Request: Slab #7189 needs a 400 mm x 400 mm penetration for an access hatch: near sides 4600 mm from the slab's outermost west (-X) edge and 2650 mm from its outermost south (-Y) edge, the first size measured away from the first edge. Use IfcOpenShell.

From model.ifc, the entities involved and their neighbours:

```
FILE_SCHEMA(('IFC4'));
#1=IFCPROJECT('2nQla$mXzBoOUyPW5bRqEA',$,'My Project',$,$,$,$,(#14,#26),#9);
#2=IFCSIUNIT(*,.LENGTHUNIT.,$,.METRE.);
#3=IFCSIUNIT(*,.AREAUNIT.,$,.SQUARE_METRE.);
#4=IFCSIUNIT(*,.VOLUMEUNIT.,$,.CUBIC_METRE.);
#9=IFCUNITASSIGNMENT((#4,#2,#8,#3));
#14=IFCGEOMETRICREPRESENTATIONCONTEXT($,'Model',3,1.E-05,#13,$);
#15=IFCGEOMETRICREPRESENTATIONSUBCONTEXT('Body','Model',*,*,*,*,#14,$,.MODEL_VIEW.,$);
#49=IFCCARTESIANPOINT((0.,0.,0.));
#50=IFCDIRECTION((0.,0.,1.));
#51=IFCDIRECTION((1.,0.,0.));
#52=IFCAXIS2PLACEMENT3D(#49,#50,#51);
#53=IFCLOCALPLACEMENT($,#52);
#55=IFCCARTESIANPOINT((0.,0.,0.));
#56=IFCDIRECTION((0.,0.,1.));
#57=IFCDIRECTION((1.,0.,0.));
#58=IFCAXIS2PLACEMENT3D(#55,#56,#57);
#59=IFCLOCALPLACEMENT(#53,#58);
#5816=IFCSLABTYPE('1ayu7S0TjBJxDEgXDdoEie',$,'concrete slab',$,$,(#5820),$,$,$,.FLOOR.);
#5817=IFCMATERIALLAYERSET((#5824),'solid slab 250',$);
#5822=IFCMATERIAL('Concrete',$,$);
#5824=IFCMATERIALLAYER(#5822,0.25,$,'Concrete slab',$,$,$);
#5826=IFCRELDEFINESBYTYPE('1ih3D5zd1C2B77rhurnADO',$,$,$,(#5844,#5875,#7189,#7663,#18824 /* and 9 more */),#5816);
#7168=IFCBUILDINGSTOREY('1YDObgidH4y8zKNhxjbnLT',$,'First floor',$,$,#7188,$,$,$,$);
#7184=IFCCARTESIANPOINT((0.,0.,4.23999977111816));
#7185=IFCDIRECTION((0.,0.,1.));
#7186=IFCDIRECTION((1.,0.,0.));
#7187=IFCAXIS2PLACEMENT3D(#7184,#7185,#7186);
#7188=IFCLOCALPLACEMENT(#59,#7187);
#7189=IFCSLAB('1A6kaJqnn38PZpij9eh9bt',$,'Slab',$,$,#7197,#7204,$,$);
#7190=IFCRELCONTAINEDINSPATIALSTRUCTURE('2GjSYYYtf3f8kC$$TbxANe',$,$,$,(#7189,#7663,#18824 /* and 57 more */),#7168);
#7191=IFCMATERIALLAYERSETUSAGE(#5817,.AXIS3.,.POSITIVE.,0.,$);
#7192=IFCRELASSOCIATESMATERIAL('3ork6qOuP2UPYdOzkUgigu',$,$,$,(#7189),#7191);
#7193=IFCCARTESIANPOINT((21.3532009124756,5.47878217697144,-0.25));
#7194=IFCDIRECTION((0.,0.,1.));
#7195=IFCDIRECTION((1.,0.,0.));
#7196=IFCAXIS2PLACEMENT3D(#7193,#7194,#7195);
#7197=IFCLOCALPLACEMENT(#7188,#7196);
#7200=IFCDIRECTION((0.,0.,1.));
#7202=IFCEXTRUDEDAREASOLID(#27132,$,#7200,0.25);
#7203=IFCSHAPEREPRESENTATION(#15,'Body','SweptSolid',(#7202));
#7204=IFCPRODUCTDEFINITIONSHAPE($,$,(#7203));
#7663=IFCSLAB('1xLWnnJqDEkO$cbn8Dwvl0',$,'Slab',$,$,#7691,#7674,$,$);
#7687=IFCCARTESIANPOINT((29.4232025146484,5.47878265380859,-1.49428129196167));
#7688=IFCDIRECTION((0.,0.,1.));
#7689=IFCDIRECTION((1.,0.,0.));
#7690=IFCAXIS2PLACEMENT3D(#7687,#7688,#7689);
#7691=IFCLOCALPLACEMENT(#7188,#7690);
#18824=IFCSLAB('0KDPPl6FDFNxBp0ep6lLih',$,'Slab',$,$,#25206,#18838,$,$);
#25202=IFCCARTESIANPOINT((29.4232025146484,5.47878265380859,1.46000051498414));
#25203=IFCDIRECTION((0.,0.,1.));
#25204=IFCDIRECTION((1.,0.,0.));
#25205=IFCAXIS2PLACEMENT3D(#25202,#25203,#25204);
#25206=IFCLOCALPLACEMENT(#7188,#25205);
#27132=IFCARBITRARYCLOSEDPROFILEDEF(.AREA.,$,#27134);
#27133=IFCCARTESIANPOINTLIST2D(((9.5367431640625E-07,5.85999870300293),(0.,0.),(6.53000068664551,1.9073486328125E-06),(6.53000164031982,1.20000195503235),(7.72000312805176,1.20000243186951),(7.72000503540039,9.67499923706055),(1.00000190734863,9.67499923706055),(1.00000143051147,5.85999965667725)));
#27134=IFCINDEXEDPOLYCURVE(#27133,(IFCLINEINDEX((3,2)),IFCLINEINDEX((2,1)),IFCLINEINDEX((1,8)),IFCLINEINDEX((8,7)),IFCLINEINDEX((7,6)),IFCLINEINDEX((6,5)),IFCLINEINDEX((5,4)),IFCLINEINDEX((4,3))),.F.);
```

```python
import numpy as np
import ifcopenshell
import ifcopenshell.api.feature
import ifcopenshell.api.geometry
import ifcopenshell.api.root
import ifcopenshell.geom
import ifcopenshell.util.placement
import ifcopenshell.util.representation
import ifcopenshell.util.shape
import ifcopenshell.util.unit

model = ifcopenshell.open("model.ifc")
unit_scale = ifcopenshell.util.unit.calculate_unit_scale(model)
settings = ifcopenshell.geom.settings()


def volume(element):
    """Net volume in cubic metres, openings subtracted."""
    shape = ifcopenshell.geom.create_shape(settings, element)
    return ifcopenshell.util.shape.get_volume(shape.geometry)


slab = model.by_id(7189)
before = volume(slab)

# Extent in the slab's own axes, in metres. The edges named are its -X and -Y sides.
slab_shape = ifcopenshell.geom.create_shape(settings, slab)
vertices = ifcopenshell.util.shape.get_vertices(slab_shape.geometry)
x_min, y_min, bottom = vertices.min(axis=0)
top = vertices[:, 2].max()

opening = ifcopenshell.api.root.create_entity(model, ifc_class="IfcOpeningElement", name="Access hatch opening", predefined_type="OPENING")
context = ifcopenshell.util.representation.get_context(model, "Model", "Body", "MODEL_VIEW")
width, depth = 0.4, 0.4
outline = [(0.0, 0.0), (width, 0.0), (width, depth), (0.0, depth), (0.0, 0.0)]
# Overshoot both faces by 50 mm so the cut is clean.
shape = ifcopenshell.api.geometry.add_slab_representation(
    model, context=context, depth=top - bottom + 0.1, polyline=outline
)
ifcopenshell.api.geometry.assign_representation(model, product=opening, representation=shape)

matrix = ifcopenshell.util.placement.get_local_placement(slab.ObjectPlacement)
matrix[:, 3] = matrix @ np.append(np.array([x_min + 4.6, y_min + 2.65, bottom - 0.05]) / unit_scale, 1.0)
ifcopenshell.api.geometry.edit_object_placement(model, product=opening, matrix=matrix, is_si=False)
ifcopenshell.api.feature.add_feature(model, feature=opening, element=slab)

after = volume(slab)

print(f"slab volume {before:.3f} -> {after:.3f} m3")

model.write("model-out.ifc")
```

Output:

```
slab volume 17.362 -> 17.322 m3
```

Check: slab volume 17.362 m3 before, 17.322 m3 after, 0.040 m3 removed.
